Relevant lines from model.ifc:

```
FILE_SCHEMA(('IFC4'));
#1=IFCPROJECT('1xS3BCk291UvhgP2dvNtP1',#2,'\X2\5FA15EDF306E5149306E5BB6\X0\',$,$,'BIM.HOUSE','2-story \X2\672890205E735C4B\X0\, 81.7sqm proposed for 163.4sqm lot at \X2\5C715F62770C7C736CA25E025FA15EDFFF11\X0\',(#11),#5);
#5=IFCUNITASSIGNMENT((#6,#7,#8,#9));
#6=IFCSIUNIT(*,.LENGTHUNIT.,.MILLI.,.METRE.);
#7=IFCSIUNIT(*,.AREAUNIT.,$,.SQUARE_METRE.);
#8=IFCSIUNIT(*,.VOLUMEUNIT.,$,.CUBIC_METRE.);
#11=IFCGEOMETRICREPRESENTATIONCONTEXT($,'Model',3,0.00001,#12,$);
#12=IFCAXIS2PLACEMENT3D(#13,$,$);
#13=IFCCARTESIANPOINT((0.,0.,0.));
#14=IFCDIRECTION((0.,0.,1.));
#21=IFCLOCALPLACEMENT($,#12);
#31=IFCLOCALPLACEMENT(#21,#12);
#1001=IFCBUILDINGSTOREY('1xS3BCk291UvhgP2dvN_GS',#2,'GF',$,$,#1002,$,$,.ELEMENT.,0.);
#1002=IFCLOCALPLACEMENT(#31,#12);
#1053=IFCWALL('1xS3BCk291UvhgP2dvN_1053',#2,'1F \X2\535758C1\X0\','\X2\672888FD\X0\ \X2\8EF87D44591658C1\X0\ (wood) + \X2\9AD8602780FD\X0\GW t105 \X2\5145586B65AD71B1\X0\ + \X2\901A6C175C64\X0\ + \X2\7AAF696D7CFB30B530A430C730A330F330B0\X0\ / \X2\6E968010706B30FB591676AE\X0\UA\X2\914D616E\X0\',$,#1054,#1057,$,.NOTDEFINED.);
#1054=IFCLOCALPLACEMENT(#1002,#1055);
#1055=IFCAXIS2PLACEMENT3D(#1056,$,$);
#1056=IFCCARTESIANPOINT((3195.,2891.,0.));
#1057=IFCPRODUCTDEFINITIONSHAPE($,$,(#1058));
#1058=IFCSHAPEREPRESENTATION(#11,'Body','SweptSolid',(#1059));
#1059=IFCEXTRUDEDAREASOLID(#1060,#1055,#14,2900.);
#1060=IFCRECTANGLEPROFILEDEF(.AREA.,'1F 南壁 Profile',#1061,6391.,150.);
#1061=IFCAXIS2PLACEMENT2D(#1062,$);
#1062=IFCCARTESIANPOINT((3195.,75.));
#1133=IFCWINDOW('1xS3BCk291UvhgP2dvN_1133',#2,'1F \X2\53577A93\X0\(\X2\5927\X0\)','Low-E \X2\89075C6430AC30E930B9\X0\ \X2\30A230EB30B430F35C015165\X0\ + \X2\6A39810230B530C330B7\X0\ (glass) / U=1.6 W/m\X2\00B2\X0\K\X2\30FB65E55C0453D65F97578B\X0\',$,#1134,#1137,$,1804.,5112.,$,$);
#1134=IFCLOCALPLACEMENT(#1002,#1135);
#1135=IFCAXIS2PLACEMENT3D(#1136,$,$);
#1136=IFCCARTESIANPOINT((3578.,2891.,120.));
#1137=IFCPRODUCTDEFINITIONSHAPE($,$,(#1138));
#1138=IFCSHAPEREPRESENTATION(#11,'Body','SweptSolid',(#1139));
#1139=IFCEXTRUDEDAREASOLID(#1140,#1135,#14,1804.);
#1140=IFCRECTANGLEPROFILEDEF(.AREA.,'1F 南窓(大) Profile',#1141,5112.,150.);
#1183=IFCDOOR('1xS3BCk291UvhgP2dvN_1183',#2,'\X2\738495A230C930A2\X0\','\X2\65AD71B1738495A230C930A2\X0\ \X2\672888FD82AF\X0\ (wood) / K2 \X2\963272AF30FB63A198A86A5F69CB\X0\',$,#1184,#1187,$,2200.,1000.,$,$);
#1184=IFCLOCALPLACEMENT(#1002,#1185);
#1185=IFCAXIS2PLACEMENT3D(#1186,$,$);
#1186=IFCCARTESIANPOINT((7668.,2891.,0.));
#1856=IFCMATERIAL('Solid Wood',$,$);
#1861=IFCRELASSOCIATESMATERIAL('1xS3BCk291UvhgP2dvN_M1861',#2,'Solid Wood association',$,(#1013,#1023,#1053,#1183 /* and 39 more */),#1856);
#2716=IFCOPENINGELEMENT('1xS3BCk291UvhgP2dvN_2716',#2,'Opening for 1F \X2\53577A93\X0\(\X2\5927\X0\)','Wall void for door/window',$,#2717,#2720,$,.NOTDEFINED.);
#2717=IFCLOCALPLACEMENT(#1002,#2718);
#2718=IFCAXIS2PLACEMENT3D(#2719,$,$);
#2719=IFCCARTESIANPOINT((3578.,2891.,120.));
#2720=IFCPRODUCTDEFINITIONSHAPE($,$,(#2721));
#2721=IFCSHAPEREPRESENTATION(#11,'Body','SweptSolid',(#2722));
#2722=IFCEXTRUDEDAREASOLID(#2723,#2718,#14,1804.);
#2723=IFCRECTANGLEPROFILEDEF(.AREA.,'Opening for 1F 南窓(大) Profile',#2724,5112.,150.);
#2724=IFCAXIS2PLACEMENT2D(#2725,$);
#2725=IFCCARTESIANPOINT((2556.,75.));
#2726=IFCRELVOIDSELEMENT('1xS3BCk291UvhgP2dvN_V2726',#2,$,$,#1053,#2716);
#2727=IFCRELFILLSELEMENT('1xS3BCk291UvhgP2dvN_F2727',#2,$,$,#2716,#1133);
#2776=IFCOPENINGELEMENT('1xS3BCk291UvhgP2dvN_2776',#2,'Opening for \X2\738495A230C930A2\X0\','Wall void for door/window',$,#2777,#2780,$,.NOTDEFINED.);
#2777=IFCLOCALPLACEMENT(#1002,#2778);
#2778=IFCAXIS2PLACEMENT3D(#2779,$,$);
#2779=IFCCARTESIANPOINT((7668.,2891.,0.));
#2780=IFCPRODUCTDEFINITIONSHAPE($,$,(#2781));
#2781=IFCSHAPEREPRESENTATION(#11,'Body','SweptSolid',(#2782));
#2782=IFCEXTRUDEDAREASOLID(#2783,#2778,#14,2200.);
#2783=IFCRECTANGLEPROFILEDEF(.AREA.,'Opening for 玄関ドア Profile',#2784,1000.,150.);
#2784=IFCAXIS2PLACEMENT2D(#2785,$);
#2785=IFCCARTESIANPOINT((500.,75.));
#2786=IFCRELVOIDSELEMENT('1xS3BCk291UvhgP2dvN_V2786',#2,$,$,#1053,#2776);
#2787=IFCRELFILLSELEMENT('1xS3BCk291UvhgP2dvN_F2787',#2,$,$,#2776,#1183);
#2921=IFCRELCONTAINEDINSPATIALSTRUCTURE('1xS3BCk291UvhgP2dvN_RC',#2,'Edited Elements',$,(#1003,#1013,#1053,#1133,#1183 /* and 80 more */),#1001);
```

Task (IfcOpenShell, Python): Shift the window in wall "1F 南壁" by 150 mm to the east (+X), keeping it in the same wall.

```python
import ifcopenshell
import ifcopenshell.api.geometry
import ifcopenshell.util.placement
import ifcopenshell.util.unit

model = ifcopenshell.open("model.ifc")
unit_scale = ifcopenshell.util.unit.calculate_unit_scale(model)

window = model.by_guid("1xS3BCk291UvhgP2dvN_1133")
opening = window.FillsVoids[0].RelatingOpeningElement
wall = opening.VoidsElements[0].RelatingBuildingElement

wall_matrix = ifcopenshell.util.placement.get_local_placement(wall.ObjectPlacement)
shift = wall_matrix[:3, 0] * 0.15 / unit_scale
before = ifcopenshell.util.placement.get_local_placement(window.ObjectPlacement)[:3, 3].copy()

# The window is not placed relative to its opening, so move both.
for product in (opening, window):
    matrix = ifcopenshell.util.placement.get_local_placement(product.ObjectPlacement)
    matrix[:3, 3] += shift
    ifcopenshell.api.geometry.edit_object_placement(model, product=product, matrix=matrix, is_si=False)

after = ifcopenshell.util.placement.get_local_placement(window.ObjectPlacement)[:3, 3]
print("window moved by", (after - before).round(3) + 0.0)

model.write("model_rev.ifc")
```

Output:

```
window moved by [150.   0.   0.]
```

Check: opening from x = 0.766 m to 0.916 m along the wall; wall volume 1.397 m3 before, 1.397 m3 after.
